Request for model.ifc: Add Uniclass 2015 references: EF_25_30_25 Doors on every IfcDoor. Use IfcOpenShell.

First a look at what the model holds.

```python
import ifcopenshell

model = ifcopenshell.open("model.ifc")
print(model.schema)
print("classifications:", [c.Name for c in model.by_type("IfcClassification")])
for ifc_class in ("IfcDoor", "IfcRoof", "IfcStair", "IfcWall", "IfcWindow"):
    print(ifc_class, len(model.by_type(ifc_class)))
```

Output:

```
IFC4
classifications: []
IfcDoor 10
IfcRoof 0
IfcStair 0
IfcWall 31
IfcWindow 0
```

```python
import ifcopenshell
import ifcopenshell.api.classification

model = ifcopenshell.open("model.ifc")

system = ifcopenshell.api.classification.add_classification(model, classification="Uniclass 2015")

codes = {
    "IfcDoor": ("EF_25_30_25", "Doors"),
}
for ifc_class, (code, name) in codes.items():
    products = model.by_type(ifc_class)
    ifcopenshell.api.classification.add_reference(
        model, products=products, classification=system, identification=code, name=name
    )
    print(code, len(products))

model.write("model_v2.ifc")
```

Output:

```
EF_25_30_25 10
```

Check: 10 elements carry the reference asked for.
